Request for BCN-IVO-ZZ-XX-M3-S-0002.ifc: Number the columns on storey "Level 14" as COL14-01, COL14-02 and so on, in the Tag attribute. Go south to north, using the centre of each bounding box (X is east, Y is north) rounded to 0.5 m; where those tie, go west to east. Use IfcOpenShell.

First a look at what the model holds.

```python
import ifcopenshell
import ifcopenshell.util.element
import ifcopenshell.util.placement

model = ifcopenshell.open("BCN-IVO-ZZ-XX-M3-S-0002.ifc")
print(model.schema)
storey = next(s for s in model.by_type("IfcBuildingStorey") if s.Name == "Level 14")
columns = [e for e in ifcopenshell.util.element.get_decomposition(storey) if e.is_a("IfcColumn")]
for e in sorted(columns, key=lambda e: e.id()):
    origin = ifcopenshell.util.placement.get_local_placement(e.ObjectPlacement)[:3, 3]
    print(e.id(), e.Tag, e.Name, origin.round(2) + 0.0, sep=" | ")
```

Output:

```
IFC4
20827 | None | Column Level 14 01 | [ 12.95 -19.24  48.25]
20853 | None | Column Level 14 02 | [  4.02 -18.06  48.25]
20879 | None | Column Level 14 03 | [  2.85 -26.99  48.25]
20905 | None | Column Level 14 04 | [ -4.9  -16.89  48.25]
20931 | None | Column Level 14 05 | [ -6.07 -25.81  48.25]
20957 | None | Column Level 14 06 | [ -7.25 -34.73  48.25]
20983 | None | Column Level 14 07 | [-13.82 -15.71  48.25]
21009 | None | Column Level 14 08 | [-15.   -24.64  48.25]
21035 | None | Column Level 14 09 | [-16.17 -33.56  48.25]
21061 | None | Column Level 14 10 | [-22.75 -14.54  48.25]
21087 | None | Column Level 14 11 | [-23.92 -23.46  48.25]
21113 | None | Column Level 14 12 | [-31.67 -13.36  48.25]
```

```python
import ifcopenshell
import ifcopenshell.geom
import ifcopenshell.util.element
import ifcopenshell.util.shape

model = ifcopenshell.open("BCN-IVO-ZZ-XX-M3-S-0002.ifc")
settings = ifcopenshell.geom.settings()
settings.set("use-world-coords", True)


def centre(element):
    shape = ifcopenshell.geom.create_shape(settings, element)
    return ifcopenshell.util.shape.get_bbox_centroid(shape.geometry)


storey = next(s for s in model.by_type("IfcBuildingStorey") if s.Name == "Level 14")
columns = [e for e in ifcopenshell.util.element.get_decomposition(storey) if e.is_a("IfcColumn")]

# Insertion points can sit at a corner or the storey origin, so sort by the geometry (in metres).
centres = {e: centre(e) for e in columns}
columns.sort(key=lambda e: (round(centres[e][1] / 0.5), centres[e][0]))

for i, e in enumerate(columns, start=1):
    number = f"COL14-{i:02d}"
    e.Tag = number
    print(e.id(), number)

model.write("BCN-IVO-ZZ-XX-M3-S-0002_updated.ifc")
```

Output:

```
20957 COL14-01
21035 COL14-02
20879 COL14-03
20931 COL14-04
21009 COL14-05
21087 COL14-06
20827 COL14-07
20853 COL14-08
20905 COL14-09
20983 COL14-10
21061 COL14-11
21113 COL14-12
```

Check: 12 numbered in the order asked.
